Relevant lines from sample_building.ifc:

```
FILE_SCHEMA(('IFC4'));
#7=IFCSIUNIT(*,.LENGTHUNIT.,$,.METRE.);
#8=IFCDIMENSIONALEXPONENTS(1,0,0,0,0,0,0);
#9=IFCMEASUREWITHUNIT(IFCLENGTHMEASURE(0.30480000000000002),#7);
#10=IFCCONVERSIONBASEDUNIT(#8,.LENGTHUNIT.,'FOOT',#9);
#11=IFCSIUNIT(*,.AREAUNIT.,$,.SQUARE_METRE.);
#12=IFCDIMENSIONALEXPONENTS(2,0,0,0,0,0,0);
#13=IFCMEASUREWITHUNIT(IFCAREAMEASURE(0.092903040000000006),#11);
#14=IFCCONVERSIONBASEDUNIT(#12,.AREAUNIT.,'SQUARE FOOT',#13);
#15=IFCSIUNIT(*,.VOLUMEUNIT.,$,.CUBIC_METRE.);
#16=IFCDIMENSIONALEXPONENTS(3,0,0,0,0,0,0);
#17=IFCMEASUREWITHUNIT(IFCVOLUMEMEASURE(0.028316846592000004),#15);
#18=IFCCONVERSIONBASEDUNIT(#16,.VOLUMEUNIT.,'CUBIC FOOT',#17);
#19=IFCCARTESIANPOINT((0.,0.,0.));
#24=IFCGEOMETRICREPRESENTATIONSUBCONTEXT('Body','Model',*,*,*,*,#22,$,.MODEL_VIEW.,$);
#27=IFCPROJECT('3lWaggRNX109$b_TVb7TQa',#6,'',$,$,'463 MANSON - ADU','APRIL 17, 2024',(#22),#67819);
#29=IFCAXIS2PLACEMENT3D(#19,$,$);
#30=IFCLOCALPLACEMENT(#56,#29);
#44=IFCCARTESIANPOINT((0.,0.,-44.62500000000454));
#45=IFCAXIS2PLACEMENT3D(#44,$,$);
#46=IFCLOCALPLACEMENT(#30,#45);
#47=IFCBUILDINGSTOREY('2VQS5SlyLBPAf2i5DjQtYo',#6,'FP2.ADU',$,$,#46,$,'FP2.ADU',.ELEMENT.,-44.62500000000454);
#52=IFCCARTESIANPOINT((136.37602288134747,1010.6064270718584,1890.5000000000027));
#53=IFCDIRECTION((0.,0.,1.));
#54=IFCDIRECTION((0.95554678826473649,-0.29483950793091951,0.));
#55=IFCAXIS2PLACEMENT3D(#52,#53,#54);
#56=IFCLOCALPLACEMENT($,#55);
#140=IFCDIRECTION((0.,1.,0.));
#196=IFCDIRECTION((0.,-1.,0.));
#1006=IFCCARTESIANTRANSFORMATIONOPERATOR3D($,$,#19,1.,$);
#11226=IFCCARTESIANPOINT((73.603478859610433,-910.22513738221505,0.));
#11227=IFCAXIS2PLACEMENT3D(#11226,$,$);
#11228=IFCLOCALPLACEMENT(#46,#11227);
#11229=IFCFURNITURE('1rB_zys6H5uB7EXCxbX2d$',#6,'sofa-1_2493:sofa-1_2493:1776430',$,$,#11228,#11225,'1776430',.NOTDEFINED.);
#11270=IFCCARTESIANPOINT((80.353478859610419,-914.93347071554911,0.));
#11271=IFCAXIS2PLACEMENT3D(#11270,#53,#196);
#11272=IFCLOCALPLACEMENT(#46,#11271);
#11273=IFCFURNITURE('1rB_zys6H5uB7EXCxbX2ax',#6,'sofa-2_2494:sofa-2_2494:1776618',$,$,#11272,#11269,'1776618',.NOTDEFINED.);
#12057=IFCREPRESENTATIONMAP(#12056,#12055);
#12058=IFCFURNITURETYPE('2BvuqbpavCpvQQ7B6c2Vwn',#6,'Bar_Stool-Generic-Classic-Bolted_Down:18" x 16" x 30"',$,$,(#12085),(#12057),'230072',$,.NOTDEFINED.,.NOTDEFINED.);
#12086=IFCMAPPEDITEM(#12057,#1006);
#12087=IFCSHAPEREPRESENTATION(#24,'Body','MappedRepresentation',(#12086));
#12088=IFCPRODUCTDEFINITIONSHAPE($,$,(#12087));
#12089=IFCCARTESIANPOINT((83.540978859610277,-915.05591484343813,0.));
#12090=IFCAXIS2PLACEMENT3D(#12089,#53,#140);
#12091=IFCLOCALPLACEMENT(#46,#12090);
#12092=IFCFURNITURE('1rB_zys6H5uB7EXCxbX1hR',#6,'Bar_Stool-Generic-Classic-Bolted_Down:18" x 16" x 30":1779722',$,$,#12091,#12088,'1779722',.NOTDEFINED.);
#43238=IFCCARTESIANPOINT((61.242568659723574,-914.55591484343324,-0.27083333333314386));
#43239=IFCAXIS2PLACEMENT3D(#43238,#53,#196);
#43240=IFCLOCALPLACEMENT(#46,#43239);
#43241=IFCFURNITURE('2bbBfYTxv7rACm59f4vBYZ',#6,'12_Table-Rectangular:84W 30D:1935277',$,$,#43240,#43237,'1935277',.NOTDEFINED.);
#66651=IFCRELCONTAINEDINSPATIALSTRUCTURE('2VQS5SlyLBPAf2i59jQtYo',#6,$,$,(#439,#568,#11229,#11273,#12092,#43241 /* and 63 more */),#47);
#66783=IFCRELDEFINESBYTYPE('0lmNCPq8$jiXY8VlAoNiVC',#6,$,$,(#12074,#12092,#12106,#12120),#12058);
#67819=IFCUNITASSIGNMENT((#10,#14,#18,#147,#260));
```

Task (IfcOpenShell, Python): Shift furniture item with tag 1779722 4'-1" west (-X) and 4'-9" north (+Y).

```python
import ifcopenshell
import ifcopenshell.api.geometry
import ifcopenshell.util.placement
import ifcopenshell.util.unit

model = ifcopenshell.open("sample_building.ifc")
unit_scale = ifcopenshell.util.unit.calculate_unit_scale(model)

item = model.by_guid("1rB_zys6H5uB7EXCxbX1hR")
matrix = ifcopenshell.util.placement.get_local_placement(item.ObjectPlacement)
matrix[0, 3] -= 49 * 0.0254 / unit_scale
matrix[1, 3] += 57 * 0.0254 / unit_scale
ifcopenshell.api.geometry.edit_object_placement(model, product=item, matrix=matrix, is_si=False)

print(ifcopenshell.util.placement.get_local_placement(item.ObjectPlacement).round(3) + 0.0)

model.write("sample_building_edited.ifc")
```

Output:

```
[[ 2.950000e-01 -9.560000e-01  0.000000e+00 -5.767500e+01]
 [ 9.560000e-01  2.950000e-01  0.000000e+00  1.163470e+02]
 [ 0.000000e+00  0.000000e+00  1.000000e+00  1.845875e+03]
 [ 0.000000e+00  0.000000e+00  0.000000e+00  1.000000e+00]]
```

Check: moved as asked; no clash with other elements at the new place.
